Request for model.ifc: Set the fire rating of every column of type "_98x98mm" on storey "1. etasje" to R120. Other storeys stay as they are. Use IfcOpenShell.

First a look at what the model holds.

```python
import ifcopenshell
import ifcopenshell.util.element

model = ifcopenshell.open("model.ifc")
print(model.schema)
storey = next(s for s in model.by_type("IfcBuildingStorey") if s.Name == "1. etasje")
columns = [e for e in ifcopenshell.util.element.get_decomposition(storey) if e.is_a("IfcColumn")]
seen = {}
for e in columns:
    element_type = ifcopenshell.util.element.get_type(e)
    key = (element_type.Name if element_type != e and element_type else None, ifcopenshell.util.element.get_pset(e, "Pset_ColumnCommon", "FireRating"))
    seen[key] = seen.get(key, 0) + 1
for (name, value), count in sorted(seen.items(), key=str):
    print(count, "x", name, "|", value)
```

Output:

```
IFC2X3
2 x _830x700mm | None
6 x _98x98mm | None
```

```python
import ifcopenshell
import ifcopenshell.api.pset
import ifcopenshell.util.element

model = ifcopenshell.open("model.ifc")

storey = next(s for s in model.by_type("IfcBuildingStorey") if s.Name == "1. etasje")
columns = [e for e in ifcopenshell.util.element.get_decomposition(storey) if e.is_a("IfcColumn")]

count = 0
for e in columns:
    element_type = ifcopenshell.util.element.get_type(e)
    if element_type in (None, e) or element_type.Name != "_98x98mm":
        continue
    # add_pset returns the element's existing set when there is one.
    pset = ifcopenshell.api.pset.add_pset(model, product=e, name="Pset_ColumnCommon")
    ifcopenshell.api.pset.edit_pset(model, pset=pset, properties={"FireRating": "R120"})
    count += 1

print(count, "columns updated")

model.write("model-out.ifc")
```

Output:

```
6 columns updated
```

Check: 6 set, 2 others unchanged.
